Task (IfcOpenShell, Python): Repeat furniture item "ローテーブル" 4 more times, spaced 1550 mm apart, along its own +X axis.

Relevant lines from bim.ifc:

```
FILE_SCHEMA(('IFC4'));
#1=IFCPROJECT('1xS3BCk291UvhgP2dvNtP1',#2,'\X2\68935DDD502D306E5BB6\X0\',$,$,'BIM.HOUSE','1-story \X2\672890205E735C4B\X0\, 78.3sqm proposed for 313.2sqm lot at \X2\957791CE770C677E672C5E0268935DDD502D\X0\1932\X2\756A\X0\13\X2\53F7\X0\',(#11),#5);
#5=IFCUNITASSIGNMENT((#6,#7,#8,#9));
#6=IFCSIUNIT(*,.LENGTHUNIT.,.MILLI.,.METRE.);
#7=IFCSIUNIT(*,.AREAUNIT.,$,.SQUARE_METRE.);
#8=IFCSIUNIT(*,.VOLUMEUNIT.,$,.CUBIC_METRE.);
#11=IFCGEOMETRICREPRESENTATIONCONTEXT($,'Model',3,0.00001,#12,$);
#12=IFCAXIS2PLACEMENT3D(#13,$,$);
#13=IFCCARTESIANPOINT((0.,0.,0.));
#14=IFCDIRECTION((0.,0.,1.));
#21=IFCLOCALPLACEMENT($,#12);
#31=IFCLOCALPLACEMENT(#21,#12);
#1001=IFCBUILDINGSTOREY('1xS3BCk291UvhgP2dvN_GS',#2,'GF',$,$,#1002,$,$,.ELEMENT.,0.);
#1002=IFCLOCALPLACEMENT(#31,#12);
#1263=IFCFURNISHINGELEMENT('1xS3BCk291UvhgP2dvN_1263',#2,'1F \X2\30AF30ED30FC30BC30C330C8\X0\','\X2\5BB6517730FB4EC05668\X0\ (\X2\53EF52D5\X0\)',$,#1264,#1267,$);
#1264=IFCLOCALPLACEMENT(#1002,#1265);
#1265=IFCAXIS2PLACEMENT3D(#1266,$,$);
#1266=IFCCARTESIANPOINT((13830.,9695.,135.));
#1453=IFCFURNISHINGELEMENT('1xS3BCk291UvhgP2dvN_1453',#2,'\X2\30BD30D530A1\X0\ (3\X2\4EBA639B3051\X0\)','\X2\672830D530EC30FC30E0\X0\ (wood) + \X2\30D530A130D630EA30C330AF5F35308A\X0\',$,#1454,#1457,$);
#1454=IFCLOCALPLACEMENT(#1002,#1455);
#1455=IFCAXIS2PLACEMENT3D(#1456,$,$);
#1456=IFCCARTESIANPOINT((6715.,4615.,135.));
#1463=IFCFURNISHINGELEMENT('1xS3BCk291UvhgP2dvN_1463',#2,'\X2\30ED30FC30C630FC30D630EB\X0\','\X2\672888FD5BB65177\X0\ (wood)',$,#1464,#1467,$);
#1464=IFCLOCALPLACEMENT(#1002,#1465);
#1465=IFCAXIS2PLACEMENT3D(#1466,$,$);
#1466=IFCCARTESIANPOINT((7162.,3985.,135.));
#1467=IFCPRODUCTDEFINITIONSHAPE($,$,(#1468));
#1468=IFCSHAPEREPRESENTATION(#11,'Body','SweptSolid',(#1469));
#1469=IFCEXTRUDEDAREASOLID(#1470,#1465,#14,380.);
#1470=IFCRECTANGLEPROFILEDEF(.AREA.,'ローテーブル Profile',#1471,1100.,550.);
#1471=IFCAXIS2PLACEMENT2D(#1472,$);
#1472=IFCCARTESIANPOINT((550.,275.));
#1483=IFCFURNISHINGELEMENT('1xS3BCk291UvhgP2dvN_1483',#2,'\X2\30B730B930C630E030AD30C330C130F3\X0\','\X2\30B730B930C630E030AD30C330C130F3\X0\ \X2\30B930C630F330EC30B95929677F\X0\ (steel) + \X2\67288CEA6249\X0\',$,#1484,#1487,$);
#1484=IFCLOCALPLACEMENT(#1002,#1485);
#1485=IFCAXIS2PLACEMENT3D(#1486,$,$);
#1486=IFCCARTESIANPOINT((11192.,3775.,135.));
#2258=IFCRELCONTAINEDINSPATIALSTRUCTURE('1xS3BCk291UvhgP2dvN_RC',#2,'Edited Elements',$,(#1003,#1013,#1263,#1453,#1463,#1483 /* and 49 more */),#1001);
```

```python
import ifcopenshell
import ifcopenshell.api.geometry
import ifcopenshell.api.root
import ifcopenshell.util.element
import ifcopenshell.util.placement

model = ifcopenshell.open("bim.ifc")


def reuse_history(source, copy):
    """copy_class also copies each property set's owner history, people and application; keep the originals."""
    for rel in copy.IsDefinedBy:
        if rel.is_a("IfcRelDefinesByProperties") and (history := rel.RelatingPropertyDefinition.OwnerHistory):
            rel.RelatingPropertyDefinition.OwnerHistory = source.OwnerHistory
            ifcopenshell.util.element.remove_deep2(model, history)


source = model.by_id(1463)
base = ifcopenshell.util.placement.get_local_placement(source.ObjectPlacement)
step = base[:3, 0] * 1550.0

for i in range(1, 5):
    copy = ifcopenshell.api.root.copy_class(model, product=source)
    copy.Representation = ifcopenshell.util.element.copy_deep(
        model, source.Representation, exclude=["IfcGeometricRepresentationContext", "IfcRepresentationMap"]
    )
    reuse_history(source, copy)
    matrix = base.copy()
    matrix[:3, 3] += i * step
    print("added at", matrix[:3, 3].round(3) + 0.0)
    ifcopenshell.api.geometry.edit_object_placement(model, product=copy, matrix=matrix, is_si=False)

model.write("bim_edited.ifc")
```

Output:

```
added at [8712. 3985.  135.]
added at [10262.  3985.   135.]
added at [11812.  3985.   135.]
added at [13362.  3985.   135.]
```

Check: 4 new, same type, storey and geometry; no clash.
